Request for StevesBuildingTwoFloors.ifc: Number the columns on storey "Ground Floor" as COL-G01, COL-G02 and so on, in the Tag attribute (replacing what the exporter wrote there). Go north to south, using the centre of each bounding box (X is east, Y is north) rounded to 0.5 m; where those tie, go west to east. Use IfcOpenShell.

First a look at what the model holds.

```python
import ifcopenshell
import ifcopenshell.util.element
import ifcopenshell.util.placement

model = ifcopenshell.open("StevesBuildingTwoFloors.ifc")
print(model.schema)
storey = next(s for s in model.by_type("IfcBuildingStorey") if s.Name == "Ground Floor")
columns = [e for e in ifcopenshell.util.element.get_decomposition(storey) if e.is_a("IfcColumn")]
for e in sorted(columns, key=lambda e: e.id()):
    origin = ifcopenshell.util.placement.get_local_placement(e.ObjectPlacement)[:3, 3]
    print(e.id(), e.Tag, e.Name, origin.round(2) + 0.0, sep=" | ")
```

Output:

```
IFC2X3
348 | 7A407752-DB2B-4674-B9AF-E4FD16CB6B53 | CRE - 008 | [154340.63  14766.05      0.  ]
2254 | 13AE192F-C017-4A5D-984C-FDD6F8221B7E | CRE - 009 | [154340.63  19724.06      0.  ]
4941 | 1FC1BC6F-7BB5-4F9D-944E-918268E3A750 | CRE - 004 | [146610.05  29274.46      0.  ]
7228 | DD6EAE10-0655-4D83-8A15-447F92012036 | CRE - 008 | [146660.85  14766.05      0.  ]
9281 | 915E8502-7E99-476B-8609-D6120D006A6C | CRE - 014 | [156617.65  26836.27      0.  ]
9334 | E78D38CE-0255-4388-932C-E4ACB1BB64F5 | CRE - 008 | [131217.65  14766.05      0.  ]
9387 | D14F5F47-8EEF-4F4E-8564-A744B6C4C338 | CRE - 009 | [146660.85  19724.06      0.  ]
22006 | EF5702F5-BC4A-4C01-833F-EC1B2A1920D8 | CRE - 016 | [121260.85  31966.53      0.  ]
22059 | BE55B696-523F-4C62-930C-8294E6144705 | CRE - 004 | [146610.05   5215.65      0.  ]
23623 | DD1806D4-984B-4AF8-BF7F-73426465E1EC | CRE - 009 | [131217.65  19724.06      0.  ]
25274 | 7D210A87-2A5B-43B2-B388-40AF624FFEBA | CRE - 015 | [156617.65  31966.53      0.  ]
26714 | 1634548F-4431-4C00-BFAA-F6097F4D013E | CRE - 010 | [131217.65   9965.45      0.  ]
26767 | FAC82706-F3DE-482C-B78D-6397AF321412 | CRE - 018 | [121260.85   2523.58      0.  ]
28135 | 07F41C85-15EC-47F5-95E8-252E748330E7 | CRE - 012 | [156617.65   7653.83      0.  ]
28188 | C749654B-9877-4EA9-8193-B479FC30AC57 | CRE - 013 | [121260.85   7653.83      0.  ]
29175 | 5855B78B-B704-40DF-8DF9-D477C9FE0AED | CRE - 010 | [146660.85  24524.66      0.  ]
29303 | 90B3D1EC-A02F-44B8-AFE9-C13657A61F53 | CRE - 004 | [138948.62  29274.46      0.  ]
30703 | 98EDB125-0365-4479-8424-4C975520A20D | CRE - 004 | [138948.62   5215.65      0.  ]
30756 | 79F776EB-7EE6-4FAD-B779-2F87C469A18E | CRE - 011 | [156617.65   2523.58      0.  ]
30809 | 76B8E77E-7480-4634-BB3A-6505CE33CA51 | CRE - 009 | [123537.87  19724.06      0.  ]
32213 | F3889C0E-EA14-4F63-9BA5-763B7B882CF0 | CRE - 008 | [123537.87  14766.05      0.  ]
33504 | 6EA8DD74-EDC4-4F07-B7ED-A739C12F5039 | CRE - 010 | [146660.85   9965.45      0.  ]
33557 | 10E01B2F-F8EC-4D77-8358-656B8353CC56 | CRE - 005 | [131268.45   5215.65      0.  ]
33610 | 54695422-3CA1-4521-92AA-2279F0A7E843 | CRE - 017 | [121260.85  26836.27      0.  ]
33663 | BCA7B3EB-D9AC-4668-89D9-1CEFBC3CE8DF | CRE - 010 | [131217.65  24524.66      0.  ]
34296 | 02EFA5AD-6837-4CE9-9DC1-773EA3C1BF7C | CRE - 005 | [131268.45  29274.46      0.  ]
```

```python
import ifcopenshell
import ifcopenshell.geom
import ifcopenshell.util.element
import ifcopenshell.util.shape

model = ifcopenshell.open("StevesBuildingTwoFloors.ifc")
settings = ifcopenshell.geom.settings()
settings.set("use-world-coords", True)


def centre(element):
    shape = ifcopenshell.geom.create_shape(settings, element)
    return ifcopenshell.util.shape.get_bbox_centroid(shape.geometry)


storey = next(s for s in model.by_type("IfcBuildingStorey") if s.Name == "Ground Floor")
columns = [e for e in ifcopenshell.util.element.get_decomposition(storey) if e.is_a("IfcColumn")]

# Insertion points can sit at a corner or the storey origin, so sort by the geometry (in metres).
centres = {e: centre(e) for e in columns}
columns.sort(key=lambda e: (-round(centres[e][1] / 0.5), centres[e][0]))

for i, e in enumerate(columns, start=1):
    number = f"COL-G{i:02d}"
    e.Tag = number
    print(e.id(), number)

model.write("StevesBuildingTwoFloors_edited.ifc")
```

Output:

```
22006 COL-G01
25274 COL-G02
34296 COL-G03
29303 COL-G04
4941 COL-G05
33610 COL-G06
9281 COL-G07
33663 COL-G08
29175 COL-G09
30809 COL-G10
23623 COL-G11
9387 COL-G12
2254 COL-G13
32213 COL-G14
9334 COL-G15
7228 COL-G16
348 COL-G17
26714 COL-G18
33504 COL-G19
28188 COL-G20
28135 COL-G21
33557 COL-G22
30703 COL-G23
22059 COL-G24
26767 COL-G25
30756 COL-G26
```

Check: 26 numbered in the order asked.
